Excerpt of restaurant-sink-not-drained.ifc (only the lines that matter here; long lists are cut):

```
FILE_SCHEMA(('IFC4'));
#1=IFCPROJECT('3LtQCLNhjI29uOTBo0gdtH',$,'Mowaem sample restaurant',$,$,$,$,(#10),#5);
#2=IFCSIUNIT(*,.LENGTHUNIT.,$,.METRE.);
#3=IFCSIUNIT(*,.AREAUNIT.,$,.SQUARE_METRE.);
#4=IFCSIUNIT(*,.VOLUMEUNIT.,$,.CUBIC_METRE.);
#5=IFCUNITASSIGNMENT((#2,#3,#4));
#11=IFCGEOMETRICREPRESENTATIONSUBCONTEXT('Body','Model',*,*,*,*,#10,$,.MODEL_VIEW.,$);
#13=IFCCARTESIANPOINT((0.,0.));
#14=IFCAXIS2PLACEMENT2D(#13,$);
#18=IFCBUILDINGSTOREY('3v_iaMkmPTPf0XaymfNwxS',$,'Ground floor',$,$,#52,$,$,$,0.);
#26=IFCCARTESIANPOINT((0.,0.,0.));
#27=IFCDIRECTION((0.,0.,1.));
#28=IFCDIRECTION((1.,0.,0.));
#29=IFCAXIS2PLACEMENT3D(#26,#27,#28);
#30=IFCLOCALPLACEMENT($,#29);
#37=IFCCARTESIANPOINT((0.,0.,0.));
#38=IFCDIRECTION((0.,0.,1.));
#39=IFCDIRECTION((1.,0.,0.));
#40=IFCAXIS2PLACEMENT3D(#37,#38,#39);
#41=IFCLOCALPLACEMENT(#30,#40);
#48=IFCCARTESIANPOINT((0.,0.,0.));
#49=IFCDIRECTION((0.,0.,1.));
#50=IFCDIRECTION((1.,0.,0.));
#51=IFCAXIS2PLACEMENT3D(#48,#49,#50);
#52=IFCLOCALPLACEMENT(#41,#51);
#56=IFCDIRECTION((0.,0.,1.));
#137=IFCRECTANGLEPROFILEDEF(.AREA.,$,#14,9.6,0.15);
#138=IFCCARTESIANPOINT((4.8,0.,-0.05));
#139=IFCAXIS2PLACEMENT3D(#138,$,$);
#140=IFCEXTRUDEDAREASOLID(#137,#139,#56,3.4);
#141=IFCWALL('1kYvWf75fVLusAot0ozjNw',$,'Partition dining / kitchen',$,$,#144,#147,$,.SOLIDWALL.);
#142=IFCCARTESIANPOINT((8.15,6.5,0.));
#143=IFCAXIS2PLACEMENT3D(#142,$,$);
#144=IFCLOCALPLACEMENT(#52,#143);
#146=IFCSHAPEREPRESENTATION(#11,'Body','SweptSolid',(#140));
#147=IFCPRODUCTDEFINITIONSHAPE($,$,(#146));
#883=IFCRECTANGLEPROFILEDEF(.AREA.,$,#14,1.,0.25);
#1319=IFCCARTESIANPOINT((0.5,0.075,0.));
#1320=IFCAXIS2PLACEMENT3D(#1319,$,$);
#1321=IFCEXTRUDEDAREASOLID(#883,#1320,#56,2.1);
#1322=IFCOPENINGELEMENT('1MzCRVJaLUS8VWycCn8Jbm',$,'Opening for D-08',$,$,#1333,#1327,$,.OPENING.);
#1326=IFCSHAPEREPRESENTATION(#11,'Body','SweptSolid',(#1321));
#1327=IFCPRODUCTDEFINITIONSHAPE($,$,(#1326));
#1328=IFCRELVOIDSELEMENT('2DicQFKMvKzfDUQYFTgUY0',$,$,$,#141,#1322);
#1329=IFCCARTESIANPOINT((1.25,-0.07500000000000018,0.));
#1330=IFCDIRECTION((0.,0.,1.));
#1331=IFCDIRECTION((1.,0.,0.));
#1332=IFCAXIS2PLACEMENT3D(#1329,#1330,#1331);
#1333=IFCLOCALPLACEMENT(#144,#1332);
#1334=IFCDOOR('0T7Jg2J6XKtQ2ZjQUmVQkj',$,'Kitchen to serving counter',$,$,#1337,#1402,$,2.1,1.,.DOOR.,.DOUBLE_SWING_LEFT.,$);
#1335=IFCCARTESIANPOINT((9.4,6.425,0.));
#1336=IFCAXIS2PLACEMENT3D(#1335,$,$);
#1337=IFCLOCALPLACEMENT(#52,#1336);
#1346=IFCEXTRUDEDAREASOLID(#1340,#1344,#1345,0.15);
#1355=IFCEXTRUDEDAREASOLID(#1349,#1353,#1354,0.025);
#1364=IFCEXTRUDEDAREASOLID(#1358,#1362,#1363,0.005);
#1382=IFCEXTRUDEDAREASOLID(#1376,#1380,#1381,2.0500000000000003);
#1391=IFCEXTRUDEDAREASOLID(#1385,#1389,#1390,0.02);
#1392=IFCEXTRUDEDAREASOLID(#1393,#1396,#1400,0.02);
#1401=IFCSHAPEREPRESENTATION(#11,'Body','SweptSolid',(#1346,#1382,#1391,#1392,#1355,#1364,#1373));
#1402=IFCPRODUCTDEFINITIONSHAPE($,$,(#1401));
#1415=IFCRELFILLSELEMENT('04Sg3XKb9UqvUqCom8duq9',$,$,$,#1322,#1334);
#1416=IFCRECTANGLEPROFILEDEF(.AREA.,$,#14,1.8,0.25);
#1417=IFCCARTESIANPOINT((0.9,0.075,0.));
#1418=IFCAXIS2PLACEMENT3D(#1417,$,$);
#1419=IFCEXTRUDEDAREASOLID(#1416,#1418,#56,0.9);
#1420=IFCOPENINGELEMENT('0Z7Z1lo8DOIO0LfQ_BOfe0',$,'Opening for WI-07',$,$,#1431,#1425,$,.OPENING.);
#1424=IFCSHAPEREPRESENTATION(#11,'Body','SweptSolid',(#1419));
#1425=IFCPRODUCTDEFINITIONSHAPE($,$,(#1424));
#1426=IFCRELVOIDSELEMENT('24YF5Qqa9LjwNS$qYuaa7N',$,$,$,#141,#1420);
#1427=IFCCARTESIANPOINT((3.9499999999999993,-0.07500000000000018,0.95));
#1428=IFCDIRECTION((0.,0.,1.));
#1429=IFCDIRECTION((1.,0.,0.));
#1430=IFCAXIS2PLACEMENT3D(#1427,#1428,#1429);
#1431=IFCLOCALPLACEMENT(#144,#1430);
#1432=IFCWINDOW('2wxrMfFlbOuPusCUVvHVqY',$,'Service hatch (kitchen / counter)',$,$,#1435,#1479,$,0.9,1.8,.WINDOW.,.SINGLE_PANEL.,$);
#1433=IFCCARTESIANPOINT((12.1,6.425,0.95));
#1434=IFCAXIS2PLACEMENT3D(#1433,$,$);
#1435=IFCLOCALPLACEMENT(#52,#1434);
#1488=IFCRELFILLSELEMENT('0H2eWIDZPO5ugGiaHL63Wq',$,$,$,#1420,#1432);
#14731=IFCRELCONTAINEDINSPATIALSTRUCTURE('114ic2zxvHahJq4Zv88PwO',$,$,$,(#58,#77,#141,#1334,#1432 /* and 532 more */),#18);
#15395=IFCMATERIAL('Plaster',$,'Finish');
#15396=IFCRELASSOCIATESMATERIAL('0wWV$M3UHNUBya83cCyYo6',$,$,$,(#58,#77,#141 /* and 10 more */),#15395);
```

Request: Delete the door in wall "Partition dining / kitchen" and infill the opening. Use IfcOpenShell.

```python
import ifcopenshell
import ifcopenshell.api.feature
import ifcopenshell.api.root
import ifcopenshell.geom
import ifcopenshell.util.shape

model = ifcopenshell.open("restaurant-sink-not-drained.ifc")
settings = ifcopenshell.geom.settings()


def volume(element):
    """Net volume in cubic metres, openings subtracted."""
    shape = ifcopenshell.geom.create_shape(settings, element)
    return ifcopenshell.util.shape.get_volume(shape.geometry)


door = model.by_guid("0T7Jg2J6XKtQ2ZjQUmVQkj")
opening = door.FillsVoids[0].RelatingOpeningElement
wall = opening.VoidsElements[0].RelatingBuildingElement
before = volume(wall)

ifcopenshell.api.root.remove_product(model, product=door)
ifcopenshell.api.feature.remove_feature(model, feature=opening)

after = volume(wall)

print(f"wall volume {before:.3f} -> {after:.3f} m3")

model.write("restaurant-sink-not-drained-out.ifc")
```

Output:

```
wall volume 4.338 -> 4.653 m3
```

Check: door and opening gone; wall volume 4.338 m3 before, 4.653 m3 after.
